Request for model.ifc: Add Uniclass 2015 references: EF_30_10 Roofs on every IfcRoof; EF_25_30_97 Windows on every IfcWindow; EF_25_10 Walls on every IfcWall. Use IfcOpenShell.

First a look at what the model holds.

```python
import ifcopenshell

model = ifcopenshell.open("model.ifc")
print(model.schema)
print("classifications:", [c.Name for c in model.by_type("IfcClassification")])
for ifc_class in ("IfcDoor", "IfcRoof", "IfcStair", "IfcWall", "IfcWindow"):
    print(ifc_class, len(model.by_type(ifc_class)))
```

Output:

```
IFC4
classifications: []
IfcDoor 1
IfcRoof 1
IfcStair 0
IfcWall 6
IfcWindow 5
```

```python
import ifcopenshell
import ifcopenshell.api.classification

model = ifcopenshell.open("model.ifc")

system = ifcopenshell.api.classification.add_classification(model, classification="Uniclass 2015")

codes = {
    "IfcRoof": ("EF_30_10", "Roofs"),
    "IfcWindow": ("EF_25_30_97", "Windows"),
    "IfcWall": ("EF_25_10", "Walls"),
}
for ifc_class, (code, name) in codes.items():
    products = model.by_type(ifc_class)
    ifcopenshell.api.classification.add_reference(
        model, products=products, classification=system, identification=code, name=name
    )
    print(code, len(products))

model.write("model_edited.ifc")
```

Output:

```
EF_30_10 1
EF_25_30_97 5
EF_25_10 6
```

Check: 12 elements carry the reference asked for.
